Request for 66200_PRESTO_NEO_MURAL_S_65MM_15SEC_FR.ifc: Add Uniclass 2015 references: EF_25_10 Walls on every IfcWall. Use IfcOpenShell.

First a look at what the model holds.

```python
import ifcopenshell

model = ifcopenshell.open("66200_PRESTO_NEO_MURAL_S_65MM_15SEC_FR.ifc")
print(model.schema)
print("classifications:", [c.Name for c in model.by_type("IfcClassification")])
for ifc_class in ("IfcDoor", "IfcRoof", "IfcStair", "IfcWall", "IfcWindow"):
    print(ifc_class, len(model.by_type(ifc_class)))
```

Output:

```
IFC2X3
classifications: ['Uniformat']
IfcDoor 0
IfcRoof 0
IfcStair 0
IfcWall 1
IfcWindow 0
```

```python
import ifcopenshell
import ifcopenshell.api.classification

model = ifcopenshell.open("66200_PRESTO_NEO_MURAL_S_65MM_15SEC_FR.ifc")

# IFC2X3 requires Source and Edition and has no link from the project to the system.
system = model.create_entity("IfcClassification", Source="NBS", Edition="2015", Name="Uniclass 2015")

codes = {
    "IfcWall": ("EF_25_10", "Walls"),
}
for ifc_class, (code, name) in codes.items():
    products = model.by_type(ifc_class)
    ifcopenshell.api.classification.add_reference(
        model, products=products, classification=system, identification=code, name=name
    )
    print(code, len(products))

model.write("66200_PRESTO_NEO_MURAL_S_65MM_15SEC_FR_edited.ifc")
```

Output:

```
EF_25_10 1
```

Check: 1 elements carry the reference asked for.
